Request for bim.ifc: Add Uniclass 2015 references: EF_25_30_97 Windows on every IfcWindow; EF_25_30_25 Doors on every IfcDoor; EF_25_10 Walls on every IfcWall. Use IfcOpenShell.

First a look at what the model holds.

```python
import ifcopenshell

model = ifcopenshell.open("bim.ifc")
print(model.schema)
print("classifications:", [c.Name for c in model.by_type("IfcClassification")])
for ifc_class in ("IfcDoor", "IfcRoof", "IfcStair", "IfcWall", "IfcWindow"):
    print(ifc_class, len(model.by_type(ifc_class)))
```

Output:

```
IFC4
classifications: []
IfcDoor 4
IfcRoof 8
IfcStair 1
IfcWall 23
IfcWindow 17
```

```python
import ifcopenshell
import ifcopenshell.api.classification

model = ifcopenshell.open("bim.ifc")

system = ifcopenshell.api.classification.add_classification(model, classification="Uniclass 2015")

codes = {
    "IfcWindow": ("EF_25_30_97", "Windows"),
    "IfcDoor": ("EF_25_30_25", "Doors"),
    "IfcWall": ("EF_25_10", "Walls"),
}
for ifc_class, (code, name) in codes.items():
    products = model.by_type(ifc_class)
    ifcopenshell.api.classification.add_reference(
        model, products=products, classification=system, identification=code, name=name
    )
    print(code, len(products))

model.write("bim-out.ifc")
```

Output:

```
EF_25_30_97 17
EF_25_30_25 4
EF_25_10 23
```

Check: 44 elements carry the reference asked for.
